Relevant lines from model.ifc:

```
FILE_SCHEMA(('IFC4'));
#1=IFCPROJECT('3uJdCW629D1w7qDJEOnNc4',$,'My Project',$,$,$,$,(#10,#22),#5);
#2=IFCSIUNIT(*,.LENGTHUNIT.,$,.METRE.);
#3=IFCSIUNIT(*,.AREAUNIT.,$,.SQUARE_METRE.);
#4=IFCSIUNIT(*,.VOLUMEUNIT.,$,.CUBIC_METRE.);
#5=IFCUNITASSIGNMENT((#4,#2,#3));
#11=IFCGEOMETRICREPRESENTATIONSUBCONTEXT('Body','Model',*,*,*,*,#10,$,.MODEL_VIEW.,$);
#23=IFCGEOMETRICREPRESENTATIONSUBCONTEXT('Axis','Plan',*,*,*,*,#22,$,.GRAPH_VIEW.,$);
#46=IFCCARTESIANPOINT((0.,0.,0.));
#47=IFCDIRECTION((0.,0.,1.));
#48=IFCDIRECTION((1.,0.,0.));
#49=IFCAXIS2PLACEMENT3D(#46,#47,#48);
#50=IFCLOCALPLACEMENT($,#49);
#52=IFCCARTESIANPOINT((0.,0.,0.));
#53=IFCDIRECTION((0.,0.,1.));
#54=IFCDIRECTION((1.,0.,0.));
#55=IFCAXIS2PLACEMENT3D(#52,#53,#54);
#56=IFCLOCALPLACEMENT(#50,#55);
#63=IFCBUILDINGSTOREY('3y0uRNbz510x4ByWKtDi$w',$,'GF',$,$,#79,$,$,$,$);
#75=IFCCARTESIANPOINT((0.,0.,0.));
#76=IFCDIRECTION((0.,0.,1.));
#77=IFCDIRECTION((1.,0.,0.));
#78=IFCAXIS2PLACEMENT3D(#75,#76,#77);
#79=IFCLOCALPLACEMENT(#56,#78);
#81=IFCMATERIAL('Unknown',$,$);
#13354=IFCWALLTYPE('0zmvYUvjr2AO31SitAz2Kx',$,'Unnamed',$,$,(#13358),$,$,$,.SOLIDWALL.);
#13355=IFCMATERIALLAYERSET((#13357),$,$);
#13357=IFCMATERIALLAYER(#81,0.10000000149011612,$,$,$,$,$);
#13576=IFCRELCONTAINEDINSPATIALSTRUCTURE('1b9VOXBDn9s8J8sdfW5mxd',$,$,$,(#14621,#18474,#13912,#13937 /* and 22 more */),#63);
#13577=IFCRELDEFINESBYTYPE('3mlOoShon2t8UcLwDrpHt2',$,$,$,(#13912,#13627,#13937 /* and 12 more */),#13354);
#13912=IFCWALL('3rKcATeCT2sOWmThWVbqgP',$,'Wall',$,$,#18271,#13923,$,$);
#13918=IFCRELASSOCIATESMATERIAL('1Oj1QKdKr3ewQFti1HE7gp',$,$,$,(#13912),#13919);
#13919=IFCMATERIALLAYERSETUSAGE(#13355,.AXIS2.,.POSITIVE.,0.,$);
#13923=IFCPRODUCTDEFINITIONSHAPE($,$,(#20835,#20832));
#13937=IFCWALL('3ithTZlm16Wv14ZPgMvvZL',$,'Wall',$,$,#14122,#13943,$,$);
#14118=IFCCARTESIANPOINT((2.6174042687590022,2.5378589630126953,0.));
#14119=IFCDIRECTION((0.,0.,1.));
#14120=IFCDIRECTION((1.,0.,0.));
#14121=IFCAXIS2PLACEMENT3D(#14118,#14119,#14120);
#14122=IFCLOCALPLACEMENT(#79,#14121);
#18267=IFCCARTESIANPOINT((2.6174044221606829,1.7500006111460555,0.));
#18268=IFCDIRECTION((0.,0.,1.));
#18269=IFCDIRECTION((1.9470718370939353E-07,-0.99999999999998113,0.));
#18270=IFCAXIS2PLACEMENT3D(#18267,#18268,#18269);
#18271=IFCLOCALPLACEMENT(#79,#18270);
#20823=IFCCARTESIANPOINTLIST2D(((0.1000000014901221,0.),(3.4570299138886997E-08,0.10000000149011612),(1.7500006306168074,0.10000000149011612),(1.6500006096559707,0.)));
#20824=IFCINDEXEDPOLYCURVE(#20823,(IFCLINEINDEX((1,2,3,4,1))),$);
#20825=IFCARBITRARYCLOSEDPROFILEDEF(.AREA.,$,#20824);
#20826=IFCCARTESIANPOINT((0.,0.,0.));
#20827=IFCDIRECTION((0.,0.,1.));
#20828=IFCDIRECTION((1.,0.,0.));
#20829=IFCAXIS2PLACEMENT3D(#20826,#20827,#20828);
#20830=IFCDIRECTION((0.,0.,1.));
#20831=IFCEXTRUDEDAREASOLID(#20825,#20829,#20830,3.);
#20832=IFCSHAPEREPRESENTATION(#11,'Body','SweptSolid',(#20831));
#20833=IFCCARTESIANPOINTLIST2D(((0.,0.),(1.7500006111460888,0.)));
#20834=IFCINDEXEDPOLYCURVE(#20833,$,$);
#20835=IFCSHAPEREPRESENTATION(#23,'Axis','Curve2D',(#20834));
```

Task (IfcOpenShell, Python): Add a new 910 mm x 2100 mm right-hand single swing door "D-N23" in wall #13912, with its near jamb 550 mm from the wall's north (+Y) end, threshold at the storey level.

```python
import numpy as np
import ifcopenshell
import ifcopenshell.api.feature
import ifcopenshell.api.geometry
import ifcopenshell.api.root
import ifcopenshell.api.spatial
import ifcopenshell.geom
import ifcopenshell.util.element
import ifcopenshell.util.placement
import ifcopenshell.util.representation
import ifcopenshell.util.shape
import ifcopenshell.util.unit

model = ifcopenshell.open("model.ifc")
unit_scale = ifcopenshell.util.unit.calculate_unit_scale(model)
settings = ifcopenshell.geom.settings()


def volume(element):
    """Net volume in cubic metres, openings subtracted."""
    shape = ifcopenshell.geom.create_shape(settings, element)
    return ifcopenshell.util.shape.get_volume(shape.geometry)


wall = model.by_guid("3rKcATeCT2sOWmThWVbqgP")
storey = ifcopenshell.util.element.get_container(wall, ifc_class="IfcBuildingStorey")
context = ifcopenshell.util.representation.get_context(model, "Model", "Body", "MODEL_VIEW")
before = volume(wall)

width, height, from_end, sill = 0.91, 2.1, 0.55, 0.0  # metres

# The wall runs along its own X axis, and the end named is its -X end.
wall_shape = ifcopenshell.geom.create_shape(settings, wall)
x, y, z = ifcopenshell.util.shape.get_vertices(wall_shape.geometry).T
start = x.min() + from_end
face, thickness = float(y.min()), float(y.max() - y.min())
wall_matrix = ifcopenshell.util.placement.get_local_placement(wall.ObjectPlacement)
level = ifcopenshell.util.placement.get_local_placement(storey.ObjectPlacement)[2, 3]


def in_wall(x, y):
    """Placement at x, y metres in the wall's axes, at sill height."""
    matrix = wall_matrix.copy()
    matrix[:, 3] = wall_matrix @ np.array([x / unit_scale, y / unit_scale, 0.0, 1.0])
    matrix[2, 3] = level + sill / unit_scale
    return matrix


# Opening: a box that overshoots both wall faces by 50 mm.
opening = ifcopenshell.api.root.create_entity(model, ifc_class="IfcOpeningElement", predefined_type="OPENING")
box = ifcopenshell.api.geometry.add_wall_representation(
    model, context=context, length=width, height=height, thickness=thickness + 0.1
)
ifcopenshell.api.geometry.assign_representation(model, product=opening, representation=box)
ifcopenshell.api.geometry.edit_object_placement(model, product=opening, matrix=in_wall(start, face - 0.05), is_si=False)
ifcopenshell.api.feature.add_feature(model, feature=opening, element=wall)

door = ifcopenshell.api.root.create_entity(model, ifc_class="IfcDoor", name="D-N23", predefined_type="DOOR")
door.OverallWidth, door.OverallHeight = width / unit_scale, height / unit_scale
door.OperationType = "SINGLE_SWING_RIGHT"
body = ifcopenshell.api.geometry.add_door_representation(
    model,
    context=context,
    overall_width=door.OverallWidth,
    overall_height=door.OverallHeight,
    operation_type="SINGLE_SWING_RIGHT",
    lining_properties={"LiningDepth": thickness / unit_scale, "ThresholdDepth": thickness / unit_scale},
)
ifcopenshell.api.geometry.assign_representation(model, product=door, representation=body)
ifcopenshell.api.spatial.assign_container(model, products=[door], relating_structure=storey)
ifcopenshell.api.feature.add_filling(model, opening=opening, element=door)

# The lining spans the wall, so the door starts at the wall face.
ifcopenshell.api.geometry.edit_object_placement(model, product=door, matrix=in_wall(start, face), is_si=False)

after = volume(wall)

print(f"wall volume {before:.3f} -> {after:.3f} m3")

model.write("model_edited.ifc")
```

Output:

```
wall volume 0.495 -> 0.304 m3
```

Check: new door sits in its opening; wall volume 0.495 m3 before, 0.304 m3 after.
